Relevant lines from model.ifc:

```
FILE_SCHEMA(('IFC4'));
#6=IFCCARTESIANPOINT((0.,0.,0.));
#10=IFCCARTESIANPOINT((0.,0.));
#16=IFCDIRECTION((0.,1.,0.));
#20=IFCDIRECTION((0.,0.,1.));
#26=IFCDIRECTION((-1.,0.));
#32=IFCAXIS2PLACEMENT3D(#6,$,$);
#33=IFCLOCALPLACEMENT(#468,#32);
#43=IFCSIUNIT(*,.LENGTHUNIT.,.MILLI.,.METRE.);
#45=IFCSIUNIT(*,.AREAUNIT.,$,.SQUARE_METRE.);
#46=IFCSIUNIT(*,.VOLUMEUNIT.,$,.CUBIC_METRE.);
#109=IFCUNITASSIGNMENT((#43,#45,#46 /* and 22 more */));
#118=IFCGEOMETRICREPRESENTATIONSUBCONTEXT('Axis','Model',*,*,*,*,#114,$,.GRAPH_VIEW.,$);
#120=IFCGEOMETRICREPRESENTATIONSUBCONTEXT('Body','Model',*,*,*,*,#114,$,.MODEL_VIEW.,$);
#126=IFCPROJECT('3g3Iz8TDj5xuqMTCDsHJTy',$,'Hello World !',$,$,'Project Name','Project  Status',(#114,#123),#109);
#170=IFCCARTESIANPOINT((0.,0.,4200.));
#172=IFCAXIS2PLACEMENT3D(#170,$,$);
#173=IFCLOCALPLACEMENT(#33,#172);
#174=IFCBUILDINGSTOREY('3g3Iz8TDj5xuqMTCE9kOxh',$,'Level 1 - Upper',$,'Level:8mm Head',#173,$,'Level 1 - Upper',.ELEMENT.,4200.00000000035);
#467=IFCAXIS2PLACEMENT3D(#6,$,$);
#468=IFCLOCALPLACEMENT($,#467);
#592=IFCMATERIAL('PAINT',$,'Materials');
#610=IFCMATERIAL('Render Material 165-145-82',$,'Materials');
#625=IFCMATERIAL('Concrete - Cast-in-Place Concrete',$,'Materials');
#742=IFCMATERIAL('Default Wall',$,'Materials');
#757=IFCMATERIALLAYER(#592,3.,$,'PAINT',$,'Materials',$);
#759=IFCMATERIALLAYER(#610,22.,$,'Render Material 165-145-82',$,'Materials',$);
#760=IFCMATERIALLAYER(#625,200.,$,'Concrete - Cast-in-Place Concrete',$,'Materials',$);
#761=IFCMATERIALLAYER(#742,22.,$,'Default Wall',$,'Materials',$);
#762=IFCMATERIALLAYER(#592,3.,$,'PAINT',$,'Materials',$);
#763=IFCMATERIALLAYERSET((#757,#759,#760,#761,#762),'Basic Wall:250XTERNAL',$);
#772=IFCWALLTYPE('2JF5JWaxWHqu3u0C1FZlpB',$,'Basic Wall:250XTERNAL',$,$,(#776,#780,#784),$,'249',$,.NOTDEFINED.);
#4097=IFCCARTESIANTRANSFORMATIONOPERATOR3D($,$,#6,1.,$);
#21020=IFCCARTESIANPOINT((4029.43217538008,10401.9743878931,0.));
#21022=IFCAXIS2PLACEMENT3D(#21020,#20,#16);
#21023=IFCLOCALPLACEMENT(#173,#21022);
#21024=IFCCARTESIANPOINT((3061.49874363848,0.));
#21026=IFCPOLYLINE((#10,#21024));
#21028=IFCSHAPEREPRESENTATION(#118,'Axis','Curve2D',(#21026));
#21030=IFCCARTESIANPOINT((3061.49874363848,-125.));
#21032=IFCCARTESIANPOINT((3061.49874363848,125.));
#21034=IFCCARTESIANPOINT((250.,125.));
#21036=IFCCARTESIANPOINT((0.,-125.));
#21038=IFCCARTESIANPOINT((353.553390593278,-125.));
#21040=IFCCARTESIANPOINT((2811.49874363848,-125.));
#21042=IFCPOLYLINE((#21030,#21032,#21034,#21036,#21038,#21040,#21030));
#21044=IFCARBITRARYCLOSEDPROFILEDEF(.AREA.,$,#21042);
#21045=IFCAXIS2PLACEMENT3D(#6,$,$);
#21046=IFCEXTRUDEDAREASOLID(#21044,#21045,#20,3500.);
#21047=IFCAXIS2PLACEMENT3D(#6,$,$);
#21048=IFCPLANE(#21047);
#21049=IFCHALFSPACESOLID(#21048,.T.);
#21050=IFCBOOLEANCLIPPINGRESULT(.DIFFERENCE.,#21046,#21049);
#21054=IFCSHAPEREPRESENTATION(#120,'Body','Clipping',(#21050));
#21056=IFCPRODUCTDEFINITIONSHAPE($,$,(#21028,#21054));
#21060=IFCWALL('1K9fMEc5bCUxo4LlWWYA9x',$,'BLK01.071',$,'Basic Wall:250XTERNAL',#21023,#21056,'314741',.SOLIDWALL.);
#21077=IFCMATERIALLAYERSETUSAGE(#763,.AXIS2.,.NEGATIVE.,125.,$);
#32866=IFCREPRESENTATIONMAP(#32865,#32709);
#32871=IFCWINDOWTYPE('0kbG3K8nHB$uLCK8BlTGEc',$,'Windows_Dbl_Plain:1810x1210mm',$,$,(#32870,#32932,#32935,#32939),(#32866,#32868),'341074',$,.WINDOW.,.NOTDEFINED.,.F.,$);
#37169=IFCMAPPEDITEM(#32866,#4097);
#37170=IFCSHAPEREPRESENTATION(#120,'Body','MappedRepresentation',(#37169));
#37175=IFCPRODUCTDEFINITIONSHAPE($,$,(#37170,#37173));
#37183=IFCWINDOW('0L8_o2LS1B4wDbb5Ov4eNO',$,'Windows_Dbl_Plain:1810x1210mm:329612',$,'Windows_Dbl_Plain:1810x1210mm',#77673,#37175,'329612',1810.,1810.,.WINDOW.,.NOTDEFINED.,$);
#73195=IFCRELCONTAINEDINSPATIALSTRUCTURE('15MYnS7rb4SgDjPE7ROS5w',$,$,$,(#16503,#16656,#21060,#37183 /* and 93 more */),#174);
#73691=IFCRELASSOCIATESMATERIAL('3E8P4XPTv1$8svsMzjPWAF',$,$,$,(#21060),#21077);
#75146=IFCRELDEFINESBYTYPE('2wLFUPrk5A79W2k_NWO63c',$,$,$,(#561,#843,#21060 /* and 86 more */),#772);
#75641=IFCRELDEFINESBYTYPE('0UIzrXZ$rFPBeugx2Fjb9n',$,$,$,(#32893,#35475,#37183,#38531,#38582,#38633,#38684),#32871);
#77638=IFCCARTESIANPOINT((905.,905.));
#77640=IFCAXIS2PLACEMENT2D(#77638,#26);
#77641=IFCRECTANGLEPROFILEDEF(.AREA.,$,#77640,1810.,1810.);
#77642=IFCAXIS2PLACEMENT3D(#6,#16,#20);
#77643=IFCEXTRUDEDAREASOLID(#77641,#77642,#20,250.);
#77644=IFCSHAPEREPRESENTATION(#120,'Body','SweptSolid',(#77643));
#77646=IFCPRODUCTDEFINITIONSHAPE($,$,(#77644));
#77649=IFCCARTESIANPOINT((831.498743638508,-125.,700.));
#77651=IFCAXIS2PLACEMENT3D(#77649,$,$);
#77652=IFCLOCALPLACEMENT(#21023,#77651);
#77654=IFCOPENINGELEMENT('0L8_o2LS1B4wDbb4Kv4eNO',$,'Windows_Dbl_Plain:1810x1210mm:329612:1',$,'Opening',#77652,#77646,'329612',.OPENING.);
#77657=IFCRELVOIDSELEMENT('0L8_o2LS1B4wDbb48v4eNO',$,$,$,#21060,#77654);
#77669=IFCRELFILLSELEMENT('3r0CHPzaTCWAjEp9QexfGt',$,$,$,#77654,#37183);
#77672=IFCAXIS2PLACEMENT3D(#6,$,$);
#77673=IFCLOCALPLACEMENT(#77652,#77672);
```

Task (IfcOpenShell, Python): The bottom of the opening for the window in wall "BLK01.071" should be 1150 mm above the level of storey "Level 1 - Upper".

```python
import numpy as np
import ifcopenshell
import ifcopenshell.api.geometry
import ifcopenshell.geom
import ifcopenshell.util.element
import ifcopenshell.util.placement
import ifcopenshell.util.shape
import ifcopenshell.util.unit

model = ifcopenshell.open("model.ifc")
unit_scale = ifcopenshell.util.unit.calculate_unit_scale(model)

window = model.by_id(37183)
opening = window.FillsVoids[0].RelatingOpeningElement
storey = ifcopenshell.util.element.get_container(window, ifc_class="IfcBuildingStorey")
level = ifcopenshell.util.placement.get_local_placement(storey.ObjectPlacement)[2, 3]

# The opening's origin need not be at the sill, so measure its lowest point.
shape = ifcopenshell.geom.create_shape(ifcopenshell.geom.settings(), opening)
bottom = ifcopenshell.util.shape.get_shape_bottom_elevation(shape, shape.geometry) / unit_scale
dz = level + 1.15 / unit_scale - bottom

shift = np.array([0.0, 0.0, dz])
# The window is placed relative to its opening, so it follows when the opening moves.
matrix = ifcopenshell.util.placement.get_local_placement(opening.ObjectPlacement)
matrix[:3, 3] += shift
ifcopenshell.api.geometry.edit_object_placement(
    model, product=opening, matrix=matrix, is_si=False, should_transform_children=True
)

print(f"moved by {dz * unit_scale:+.3f} m")

model.write("model_v2.ifc")
```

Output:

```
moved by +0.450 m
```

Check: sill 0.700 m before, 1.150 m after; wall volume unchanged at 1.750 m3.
